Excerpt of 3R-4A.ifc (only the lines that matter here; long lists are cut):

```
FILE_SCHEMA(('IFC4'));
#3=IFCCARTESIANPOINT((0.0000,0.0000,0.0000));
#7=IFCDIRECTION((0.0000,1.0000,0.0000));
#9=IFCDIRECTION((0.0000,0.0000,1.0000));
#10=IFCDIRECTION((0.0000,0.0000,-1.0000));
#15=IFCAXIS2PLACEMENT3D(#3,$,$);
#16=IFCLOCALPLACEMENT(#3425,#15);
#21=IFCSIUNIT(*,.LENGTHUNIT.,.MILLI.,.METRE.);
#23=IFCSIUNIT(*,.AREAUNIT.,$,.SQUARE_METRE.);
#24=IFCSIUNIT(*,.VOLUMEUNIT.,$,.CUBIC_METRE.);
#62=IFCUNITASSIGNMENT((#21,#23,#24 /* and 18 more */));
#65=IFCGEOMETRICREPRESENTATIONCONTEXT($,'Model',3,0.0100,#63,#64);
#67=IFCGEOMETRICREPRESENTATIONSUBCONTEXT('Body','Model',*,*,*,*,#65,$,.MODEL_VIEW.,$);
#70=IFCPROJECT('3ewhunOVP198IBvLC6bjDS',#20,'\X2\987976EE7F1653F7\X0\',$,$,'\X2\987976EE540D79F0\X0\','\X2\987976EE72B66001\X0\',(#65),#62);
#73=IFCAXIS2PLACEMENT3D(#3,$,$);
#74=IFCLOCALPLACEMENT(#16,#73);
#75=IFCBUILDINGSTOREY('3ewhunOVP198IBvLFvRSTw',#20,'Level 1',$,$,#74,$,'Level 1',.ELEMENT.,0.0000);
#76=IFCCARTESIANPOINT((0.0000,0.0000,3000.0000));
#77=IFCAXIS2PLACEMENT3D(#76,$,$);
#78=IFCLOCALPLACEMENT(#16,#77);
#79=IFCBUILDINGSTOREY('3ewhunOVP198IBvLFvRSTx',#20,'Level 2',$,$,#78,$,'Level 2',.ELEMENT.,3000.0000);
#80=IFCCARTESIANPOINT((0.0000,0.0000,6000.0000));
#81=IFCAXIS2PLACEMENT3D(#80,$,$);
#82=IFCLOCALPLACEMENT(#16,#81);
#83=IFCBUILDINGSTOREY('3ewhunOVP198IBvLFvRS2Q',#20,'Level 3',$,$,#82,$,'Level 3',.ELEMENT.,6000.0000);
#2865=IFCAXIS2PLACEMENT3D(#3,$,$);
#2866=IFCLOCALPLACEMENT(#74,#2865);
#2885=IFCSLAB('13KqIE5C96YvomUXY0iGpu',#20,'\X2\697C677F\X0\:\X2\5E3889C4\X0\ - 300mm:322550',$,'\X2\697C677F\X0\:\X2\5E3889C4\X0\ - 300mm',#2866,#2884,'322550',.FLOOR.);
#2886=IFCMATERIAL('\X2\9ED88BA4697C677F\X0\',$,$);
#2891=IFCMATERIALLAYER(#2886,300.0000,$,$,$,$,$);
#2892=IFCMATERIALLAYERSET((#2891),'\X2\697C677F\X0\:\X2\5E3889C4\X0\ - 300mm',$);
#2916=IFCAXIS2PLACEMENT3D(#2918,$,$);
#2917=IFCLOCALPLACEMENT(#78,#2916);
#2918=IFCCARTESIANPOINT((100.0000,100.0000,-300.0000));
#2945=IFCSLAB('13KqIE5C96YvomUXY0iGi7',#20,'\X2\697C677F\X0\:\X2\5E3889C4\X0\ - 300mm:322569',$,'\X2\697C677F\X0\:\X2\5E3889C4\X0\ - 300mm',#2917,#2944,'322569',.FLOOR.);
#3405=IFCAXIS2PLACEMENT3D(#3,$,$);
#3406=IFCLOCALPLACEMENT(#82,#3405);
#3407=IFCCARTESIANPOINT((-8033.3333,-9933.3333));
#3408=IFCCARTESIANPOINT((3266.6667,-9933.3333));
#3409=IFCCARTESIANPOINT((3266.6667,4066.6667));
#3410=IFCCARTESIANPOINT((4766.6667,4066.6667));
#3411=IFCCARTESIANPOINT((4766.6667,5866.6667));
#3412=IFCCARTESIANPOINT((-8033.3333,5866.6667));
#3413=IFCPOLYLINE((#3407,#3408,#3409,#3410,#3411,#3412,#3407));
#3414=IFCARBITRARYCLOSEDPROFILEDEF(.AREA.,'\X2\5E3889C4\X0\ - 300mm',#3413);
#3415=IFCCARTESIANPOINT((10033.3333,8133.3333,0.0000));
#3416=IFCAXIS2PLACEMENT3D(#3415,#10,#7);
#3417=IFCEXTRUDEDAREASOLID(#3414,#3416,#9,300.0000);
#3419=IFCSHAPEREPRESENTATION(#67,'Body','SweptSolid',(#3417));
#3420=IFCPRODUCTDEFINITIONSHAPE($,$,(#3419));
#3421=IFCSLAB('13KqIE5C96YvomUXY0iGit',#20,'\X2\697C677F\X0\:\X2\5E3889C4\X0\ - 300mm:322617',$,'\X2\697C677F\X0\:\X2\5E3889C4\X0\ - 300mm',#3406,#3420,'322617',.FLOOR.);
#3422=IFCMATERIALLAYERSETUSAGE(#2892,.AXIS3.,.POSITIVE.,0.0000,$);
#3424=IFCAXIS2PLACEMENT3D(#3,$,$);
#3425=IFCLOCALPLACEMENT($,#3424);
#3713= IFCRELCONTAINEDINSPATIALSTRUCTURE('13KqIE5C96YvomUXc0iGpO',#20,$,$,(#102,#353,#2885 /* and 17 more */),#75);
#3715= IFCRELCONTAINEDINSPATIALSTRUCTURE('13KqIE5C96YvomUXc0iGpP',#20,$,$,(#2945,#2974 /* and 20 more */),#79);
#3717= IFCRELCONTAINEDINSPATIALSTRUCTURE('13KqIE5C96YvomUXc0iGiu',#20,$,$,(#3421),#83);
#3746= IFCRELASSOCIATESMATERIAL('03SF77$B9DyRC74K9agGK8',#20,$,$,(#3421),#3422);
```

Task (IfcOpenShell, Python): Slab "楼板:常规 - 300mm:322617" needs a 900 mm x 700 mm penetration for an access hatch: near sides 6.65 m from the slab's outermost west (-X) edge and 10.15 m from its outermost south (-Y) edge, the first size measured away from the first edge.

```python
import numpy as np
import ifcopenshell
import ifcopenshell.api.feature
import ifcopenshell.api.geometry
import ifcopenshell.api.root
import ifcopenshell.geom
import ifcopenshell.util.placement
import ifcopenshell.util.representation
import ifcopenshell.util.shape
import ifcopenshell.util.unit

model = ifcopenshell.open("3R-4A.ifc")
unit_scale = ifcopenshell.util.unit.calculate_unit_scale(model)
settings = ifcopenshell.geom.settings()


def volume(element):
    """Net volume in cubic metres, openings subtracted."""
    shape = ifcopenshell.geom.create_shape(settings, element)
    return ifcopenshell.util.shape.get_volume(shape.geometry)


slab = model.by_guid("13KqIE5C96YvomUXY0iGit")
before = volume(slab)

# Extent in the slab's own axes, in metres. The edges named are its -X and -Y sides.
slab_shape = ifcopenshell.geom.create_shape(settings, slab)
vertices = ifcopenshell.util.shape.get_vertices(slab_shape.geometry)
x_min, y_min, bottom = vertices.min(axis=0)
top = vertices[:, 2].max()

opening = ifcopenshell.api.root.create_entity(model, ifc_class="IfcOpeningElement", name="Access hatch opening", predefined_type="OPENING")
context = ifcopenshell.util.representation.get_context(model, "Model", "Body", "MODEL_VIEW")
width, depth = 0.9, 0.7
outline = [(0.0, 0.0), (width, 0.0), (width, depth), (0.0, depth), (0.0, 0.0)]
# Overshoot both faces by 50 mm so the cut is clean.
shape = ifcopenshell.api.geometry.add_slab_representation(
    model, context=context, depth=top - bottom + 0.1, polyline=outline
)
ifcopenshell.api.geometry.assign_representation(model, product=opening, representation=shape)

matrix = ifcopenshell.util.placement.get_local_placement(slab.ObjectPlacement)
matrix[:, 3] = matrix @ np.append(np.array([x_min + 6.65, y_min + 10.15, bottom - 0.05]) / unit_scale, 1.0)
ifcopenshell.api.geometry.edit_object_placement(model, product=opening, matrix=matrix, is_si=False)
ifcopenshell.api.feature.add_feature(model, feature=opening, element=slab)

after = volume(slab)

print(f"slab volume {before:.3f} -> {after:.3f} m3")

model.write("3R-4A_v2.ifc")
```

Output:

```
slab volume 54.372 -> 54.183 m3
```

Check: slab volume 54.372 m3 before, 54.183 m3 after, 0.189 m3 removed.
